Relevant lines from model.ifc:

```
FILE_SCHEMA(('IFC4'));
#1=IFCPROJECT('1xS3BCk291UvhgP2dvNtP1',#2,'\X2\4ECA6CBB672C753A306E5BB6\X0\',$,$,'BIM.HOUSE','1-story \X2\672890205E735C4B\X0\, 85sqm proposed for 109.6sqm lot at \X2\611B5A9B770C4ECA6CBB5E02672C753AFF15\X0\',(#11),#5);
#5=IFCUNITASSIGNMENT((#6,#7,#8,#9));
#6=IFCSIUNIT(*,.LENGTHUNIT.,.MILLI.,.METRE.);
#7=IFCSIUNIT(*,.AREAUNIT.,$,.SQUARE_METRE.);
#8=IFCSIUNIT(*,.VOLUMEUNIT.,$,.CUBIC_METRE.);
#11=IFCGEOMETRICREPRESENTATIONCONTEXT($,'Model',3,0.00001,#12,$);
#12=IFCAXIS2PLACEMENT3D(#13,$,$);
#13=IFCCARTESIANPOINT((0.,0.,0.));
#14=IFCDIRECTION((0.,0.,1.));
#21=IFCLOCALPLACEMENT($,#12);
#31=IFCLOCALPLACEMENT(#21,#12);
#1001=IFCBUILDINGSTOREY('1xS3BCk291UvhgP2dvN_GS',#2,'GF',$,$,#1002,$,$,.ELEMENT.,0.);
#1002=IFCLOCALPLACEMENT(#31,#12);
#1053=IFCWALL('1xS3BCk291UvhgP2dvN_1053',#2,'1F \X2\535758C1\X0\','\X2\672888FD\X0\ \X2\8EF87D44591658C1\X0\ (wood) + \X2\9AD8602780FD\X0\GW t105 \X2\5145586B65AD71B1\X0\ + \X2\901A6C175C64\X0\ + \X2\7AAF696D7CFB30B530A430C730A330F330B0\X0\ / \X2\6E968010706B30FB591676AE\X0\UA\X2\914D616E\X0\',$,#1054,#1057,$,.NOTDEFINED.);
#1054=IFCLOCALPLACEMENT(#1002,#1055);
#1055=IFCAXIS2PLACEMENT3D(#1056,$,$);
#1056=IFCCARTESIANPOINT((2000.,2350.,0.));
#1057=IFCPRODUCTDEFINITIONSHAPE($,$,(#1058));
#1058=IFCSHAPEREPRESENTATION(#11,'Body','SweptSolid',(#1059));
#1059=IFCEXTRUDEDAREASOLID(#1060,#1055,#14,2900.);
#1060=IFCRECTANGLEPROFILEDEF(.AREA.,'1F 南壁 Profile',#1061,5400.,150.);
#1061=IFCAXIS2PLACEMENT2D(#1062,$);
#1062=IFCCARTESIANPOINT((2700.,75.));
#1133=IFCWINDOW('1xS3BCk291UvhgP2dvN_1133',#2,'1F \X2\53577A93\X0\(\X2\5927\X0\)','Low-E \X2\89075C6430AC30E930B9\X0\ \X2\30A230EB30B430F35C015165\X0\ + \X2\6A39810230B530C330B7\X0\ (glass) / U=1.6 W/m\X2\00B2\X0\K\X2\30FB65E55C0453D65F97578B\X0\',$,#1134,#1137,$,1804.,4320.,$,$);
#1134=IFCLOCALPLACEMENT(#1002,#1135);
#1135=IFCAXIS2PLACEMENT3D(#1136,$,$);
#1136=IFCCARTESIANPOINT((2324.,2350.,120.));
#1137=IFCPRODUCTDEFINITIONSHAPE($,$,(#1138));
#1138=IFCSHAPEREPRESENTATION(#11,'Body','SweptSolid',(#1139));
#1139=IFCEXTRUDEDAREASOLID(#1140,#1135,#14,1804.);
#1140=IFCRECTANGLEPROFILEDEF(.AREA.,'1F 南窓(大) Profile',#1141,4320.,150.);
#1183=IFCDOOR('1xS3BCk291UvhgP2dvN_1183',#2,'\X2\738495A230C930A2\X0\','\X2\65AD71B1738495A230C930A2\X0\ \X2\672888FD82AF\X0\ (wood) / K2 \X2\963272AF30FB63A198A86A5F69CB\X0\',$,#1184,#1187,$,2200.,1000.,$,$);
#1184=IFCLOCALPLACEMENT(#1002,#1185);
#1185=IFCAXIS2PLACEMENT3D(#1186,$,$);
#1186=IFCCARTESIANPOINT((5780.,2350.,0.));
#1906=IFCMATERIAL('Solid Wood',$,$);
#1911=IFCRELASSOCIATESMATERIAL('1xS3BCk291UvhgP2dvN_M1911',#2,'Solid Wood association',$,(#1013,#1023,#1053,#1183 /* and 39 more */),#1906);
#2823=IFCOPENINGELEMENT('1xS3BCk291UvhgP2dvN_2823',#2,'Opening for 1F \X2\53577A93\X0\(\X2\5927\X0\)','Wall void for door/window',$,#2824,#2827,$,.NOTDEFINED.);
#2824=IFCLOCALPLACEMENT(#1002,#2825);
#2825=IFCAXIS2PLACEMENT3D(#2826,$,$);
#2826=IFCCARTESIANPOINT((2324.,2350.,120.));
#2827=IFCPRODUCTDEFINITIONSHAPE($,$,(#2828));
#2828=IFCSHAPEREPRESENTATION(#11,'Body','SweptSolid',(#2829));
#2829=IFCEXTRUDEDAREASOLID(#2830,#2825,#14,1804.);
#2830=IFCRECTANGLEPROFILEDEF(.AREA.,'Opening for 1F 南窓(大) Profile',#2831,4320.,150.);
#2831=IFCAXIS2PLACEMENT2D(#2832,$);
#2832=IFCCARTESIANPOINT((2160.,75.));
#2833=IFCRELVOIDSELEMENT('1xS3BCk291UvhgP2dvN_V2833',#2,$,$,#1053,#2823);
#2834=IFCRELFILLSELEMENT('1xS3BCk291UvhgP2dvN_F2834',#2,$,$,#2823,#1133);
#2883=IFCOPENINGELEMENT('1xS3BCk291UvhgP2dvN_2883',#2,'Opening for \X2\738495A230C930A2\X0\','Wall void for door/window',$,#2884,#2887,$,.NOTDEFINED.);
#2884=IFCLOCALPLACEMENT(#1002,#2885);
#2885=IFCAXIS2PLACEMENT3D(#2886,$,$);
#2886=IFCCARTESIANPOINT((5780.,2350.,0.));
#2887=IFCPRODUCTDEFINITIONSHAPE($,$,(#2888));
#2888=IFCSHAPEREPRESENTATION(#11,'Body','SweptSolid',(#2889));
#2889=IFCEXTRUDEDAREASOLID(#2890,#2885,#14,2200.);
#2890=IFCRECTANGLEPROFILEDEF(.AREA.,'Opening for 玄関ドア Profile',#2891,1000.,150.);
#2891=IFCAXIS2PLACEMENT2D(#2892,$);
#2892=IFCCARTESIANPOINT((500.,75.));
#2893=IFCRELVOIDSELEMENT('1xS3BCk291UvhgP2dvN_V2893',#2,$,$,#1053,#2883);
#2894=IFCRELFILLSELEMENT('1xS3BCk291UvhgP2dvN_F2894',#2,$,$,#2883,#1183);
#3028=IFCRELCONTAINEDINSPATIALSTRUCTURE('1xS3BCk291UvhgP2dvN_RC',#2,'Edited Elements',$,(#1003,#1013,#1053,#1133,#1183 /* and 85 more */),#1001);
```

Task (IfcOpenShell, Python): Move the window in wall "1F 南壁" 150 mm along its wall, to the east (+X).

```python
import ifcopenshell
import ifcopenshell.api.geometry
import ifcopenshell.util.placement

model = ifcopenshell.open("model.ifc")

window = model.by_guid("1xS3BCk291UvhgP2dvN_1133")
opening = window.FillsVoids[0].RelatingOpeningElement
wall = opening.VoidsElements[0].RelatingBuildingElement

wall_matrix = ifcopenshell.util.placement.get_local_placement(wall.ObjectPlacement)
shift = wall_matrix[:3, 0] * 150.0
before = ifcopenshell.util.placement.get_local_placement(window.ObjectPlacement)[:3, 3].copy()

# The window is not placed relative to its opening, so move both.
for product in (opening, window):
    matrix = ifcopenshell.util.placement.get_local_placement(product.ObjectPlacement)
    matrix[:3, 3] += shift
    ifcopenshell.api.geometry.edit_object_placement(model, product=product, matrix=matrix, is_si=False)

after = ifcopenshell.util.placement.get_local_placement(window.ObjectPlacement)[:3, 3]
print("window moved by", (after - before).round(3) + 0.0)

model.write("model-out.ifc")
```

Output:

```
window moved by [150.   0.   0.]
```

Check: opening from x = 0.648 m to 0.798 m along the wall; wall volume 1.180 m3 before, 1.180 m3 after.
